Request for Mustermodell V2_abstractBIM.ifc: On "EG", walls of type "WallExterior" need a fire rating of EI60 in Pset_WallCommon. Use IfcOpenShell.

First a look at what the model holds.

```python
import ifcopenshell
import ifcopenshell.util.element

model = ifcopenshell.open("Mustermodell V2_abstractBIM.ifc")
print(model.schema)
storey = next(s for s in model.by_type("IfcBuildingStorey") if s.Name == "EG")
walls = [e for e in ifcopenshell.util.element.get_decomposition(storey) if e.is_a("IfcWall")]
seen = {}
for e in walls:
    element_type = ifcopenshell.util.element.get_type(e)
    key = (element_type.Name if element_type != e and element_type else None, ifcopenshell.util.element.get_pset(e, "Pset_WallCommon", "FireRating"))
    seen[key] = seen.get(key, 0) + 1
for (name, value), count in sorted(seen.items(), key=str):
    print(count, "x", name, "|", value)
```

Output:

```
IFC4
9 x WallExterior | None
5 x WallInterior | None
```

```python
import ifcopenshell
import ifcopenshell.api.pset
import ifcopenshell.util.element

model = ifcopenshell.open("Mustermodell V2_abstractBIM.ifc")

storey = next(s for s in model.by_type("IfcBuildingStorey") if s.Name == "EG")
walls = [e for e in ifcopenshell.util.element.get_decomposition(storey) if e.is_a("IfcWall")]

count = 0
for e in walls:
    element_type = ifcopenshell.util.element.get_type(e)
    if element_type in (None, e) or element_type.Name != "WallExterior":
        continue
    # add_pset returns the element's existing set when there is one.
    pset = ifcopenshell.api.pset.add_pset(model, product=e, name="Pset_WallCommon")
    ifcopenshell.api.pset.edit_pset(model, pset=pset, properties={"FireRating": "EI60"})
    count += 1

print(count, "walls updated")

model.write("Mustermodell V2_abstractBIM_updated.ifc")
```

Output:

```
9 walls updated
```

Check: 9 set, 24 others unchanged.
